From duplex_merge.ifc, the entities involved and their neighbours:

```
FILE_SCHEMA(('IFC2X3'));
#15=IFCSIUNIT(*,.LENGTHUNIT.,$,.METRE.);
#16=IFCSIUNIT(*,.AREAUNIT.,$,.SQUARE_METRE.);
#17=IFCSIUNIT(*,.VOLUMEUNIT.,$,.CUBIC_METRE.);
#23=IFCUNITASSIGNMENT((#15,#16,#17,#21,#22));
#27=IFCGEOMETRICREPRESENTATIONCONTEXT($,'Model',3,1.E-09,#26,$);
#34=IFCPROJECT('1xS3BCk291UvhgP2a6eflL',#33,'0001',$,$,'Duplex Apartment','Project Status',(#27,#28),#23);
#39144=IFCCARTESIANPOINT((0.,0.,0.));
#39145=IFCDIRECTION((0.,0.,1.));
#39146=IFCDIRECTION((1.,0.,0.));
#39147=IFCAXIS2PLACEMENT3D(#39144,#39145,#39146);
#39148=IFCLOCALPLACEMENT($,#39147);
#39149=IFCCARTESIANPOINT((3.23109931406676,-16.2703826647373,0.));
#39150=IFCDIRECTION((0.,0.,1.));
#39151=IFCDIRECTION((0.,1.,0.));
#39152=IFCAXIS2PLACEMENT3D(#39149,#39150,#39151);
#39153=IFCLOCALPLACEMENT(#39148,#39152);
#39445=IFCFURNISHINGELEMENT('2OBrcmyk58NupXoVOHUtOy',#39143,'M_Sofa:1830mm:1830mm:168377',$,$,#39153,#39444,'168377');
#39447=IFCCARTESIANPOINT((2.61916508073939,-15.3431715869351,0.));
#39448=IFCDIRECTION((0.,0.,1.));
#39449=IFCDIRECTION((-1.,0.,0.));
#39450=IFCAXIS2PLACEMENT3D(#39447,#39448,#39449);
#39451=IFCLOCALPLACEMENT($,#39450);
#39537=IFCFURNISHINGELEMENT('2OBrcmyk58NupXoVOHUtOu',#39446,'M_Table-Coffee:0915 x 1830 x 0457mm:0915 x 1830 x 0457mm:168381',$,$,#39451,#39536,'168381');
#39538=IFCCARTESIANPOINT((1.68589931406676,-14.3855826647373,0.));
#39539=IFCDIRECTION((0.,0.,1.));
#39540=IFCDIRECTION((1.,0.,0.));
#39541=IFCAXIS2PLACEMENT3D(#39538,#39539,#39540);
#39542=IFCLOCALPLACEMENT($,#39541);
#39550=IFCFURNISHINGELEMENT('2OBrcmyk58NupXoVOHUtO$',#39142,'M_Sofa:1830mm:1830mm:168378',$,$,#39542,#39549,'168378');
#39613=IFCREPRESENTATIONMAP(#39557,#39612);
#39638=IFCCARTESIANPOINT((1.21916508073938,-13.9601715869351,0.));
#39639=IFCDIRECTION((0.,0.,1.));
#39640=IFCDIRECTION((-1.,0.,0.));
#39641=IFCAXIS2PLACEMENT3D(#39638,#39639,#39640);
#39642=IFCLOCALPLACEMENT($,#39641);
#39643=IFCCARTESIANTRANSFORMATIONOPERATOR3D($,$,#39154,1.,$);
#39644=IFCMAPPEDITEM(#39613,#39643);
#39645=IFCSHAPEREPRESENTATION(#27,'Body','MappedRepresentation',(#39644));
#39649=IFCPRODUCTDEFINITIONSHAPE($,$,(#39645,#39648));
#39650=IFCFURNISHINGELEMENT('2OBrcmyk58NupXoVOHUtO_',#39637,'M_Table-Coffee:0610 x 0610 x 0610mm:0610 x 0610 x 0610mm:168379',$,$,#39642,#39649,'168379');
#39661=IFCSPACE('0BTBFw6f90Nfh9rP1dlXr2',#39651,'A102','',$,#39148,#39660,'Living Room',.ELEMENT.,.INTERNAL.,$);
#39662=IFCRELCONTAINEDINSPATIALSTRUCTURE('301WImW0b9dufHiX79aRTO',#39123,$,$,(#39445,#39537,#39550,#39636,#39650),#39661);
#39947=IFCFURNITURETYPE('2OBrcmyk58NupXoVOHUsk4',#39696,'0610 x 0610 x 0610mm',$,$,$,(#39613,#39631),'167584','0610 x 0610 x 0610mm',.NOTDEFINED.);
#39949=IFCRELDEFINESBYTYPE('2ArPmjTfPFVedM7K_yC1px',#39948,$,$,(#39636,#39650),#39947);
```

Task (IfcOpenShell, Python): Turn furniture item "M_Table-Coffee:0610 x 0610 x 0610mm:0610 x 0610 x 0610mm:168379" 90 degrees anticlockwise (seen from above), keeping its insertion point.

```python
import ifcopenshell
import ifcopenshell.api.geometry
import ifcopenshell.util.placement

model = ifcopenshell.open("duplex_merge.ifc")

item = model.by_guid("2OBrcmyk58NupXoVOHUtO_")
matrix = ifcopenshell.util.placement.get_local_placement(item.ObjectPlacement)
matrix = matrix @ ifcopenshell.util.placement.rotation(90, "Z")
ifcopenshell.api.geometry.edit_object_placement(model, product=item, matrix=matrix, is_si=False)

print(ifcopenshell.util.placement.get_local_placement(item.ObjectPlacement).round(3) + 0.0)

model.write("duplex_merge_updated.ifc")
```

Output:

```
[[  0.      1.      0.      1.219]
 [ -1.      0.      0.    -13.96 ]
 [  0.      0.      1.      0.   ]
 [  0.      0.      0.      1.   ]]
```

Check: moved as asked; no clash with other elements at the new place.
